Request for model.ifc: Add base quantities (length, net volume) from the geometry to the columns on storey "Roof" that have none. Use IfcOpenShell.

First a look at what the model holds.

```python
import ifcopenshell
import ifcopenshell.util.element
import ifcopenshell.util.unit

model = ifcopenshell.open("model.ifc")
print(model.schema)
for unit_type in ("LENGTHUNIT", "AREAUNIT", "VOLUMEUNIT"):
    print(unit_type, ifcopenshell.util.unit.calculate_unit_scale(model, unit_type))
storey = next(s for s in model.by_type("IfcBuildingStorey") if s.Name == "Roof")
columns = [e for e in ifcopenshell.util.element.get_decomposition(storey) if e.is_a("IfcColumn")]
for e in sorted(columns, key=lambda e: e.id()):
    print(e.id(), e.is_a(), e.Name, list(ifcopenshell.util.element.get_psets(e, qtos_only=True)), sep=" | ")
```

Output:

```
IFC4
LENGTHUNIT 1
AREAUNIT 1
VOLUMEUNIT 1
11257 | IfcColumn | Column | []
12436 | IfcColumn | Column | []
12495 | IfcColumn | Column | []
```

```python
import ifcopenshell
import ifcopenshell.api.pset
import ifcopenshell.geom
import ifcopenshell.util.element
import ifcopenshell.util.shape
import ifcopenshell.util.unit

model = ifcopenshell.open("model.ifc")
unit_scale = ifcopenshell.util.unit.calculate_unit_scale(model)
volume_scale = ifcopenshell.util.unit.calculate_unit_scale(model, "VOLUMEUNIT")
settings = ifcopenshell.geom.settings()

storey = next(s for s in model.by_type("IfcBuildingStorey") if s.Name == "Roof")
columns = [e for e in ifcopenshell.util.element.get_decomposition(storey) if e.is_a("IfcColumn")]

for e in sorted(columns, key=lambda e: e.id()):
    if ifcopenshell.util.element.get_psets(e, qtos_only=True, should_inherit=False):
        continue
    # Geometry comes back in metres, in the element's own axes.
    shape = ifcopenshell.geom.create_shape(settings, e)
    values = {
        "Length": ifcopenshell.util.shape.get_z(shape.geometry) / unit_scale,
        "NetVolume": ifcopenshell.util.shape.get_volume(shape.geometry) / volume_scale,
    }
    qto = ifcopenshell.api.pset.add_qto(model, product=e, name="Qto_ColumnBaseQuantities")
    ifcopenshell.api.pset.edit_qto(model, qto=qto, properties=values)
    print(e.id(), {k: round(v, 3) for k, v in values.items()})

model.write("model_edited.ifc")
```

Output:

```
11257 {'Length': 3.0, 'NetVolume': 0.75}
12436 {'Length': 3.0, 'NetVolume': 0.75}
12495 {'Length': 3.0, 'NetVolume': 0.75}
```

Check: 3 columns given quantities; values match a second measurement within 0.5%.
